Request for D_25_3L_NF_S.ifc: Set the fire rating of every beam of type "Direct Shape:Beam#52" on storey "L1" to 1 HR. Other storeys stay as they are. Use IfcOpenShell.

First a look at what the model holds.

```python
import ifcopenshell
import ifcopenshell.util.element

model = ifcopenshell.open("D_25_3L_NF_S.ifc")
print(model.schema)
storey = next(s for s in model.by_type("IfcBuildingStorey") if s.Name == "L1")
beams = [e for e in ifcopenshell.util.element.get_decomposition(storey) if e.is_a("IfcBeam")]
seen = {}
for e in beams:
    element_type = ifcopenshell.util.element.get_type(e)
    key = (element_type.Name if element_type != e and element_type else None, ifcopenshell.util.element.get_pset(e, "Pset_BeamCommon", "FireRating"))
    seen[key] = seen.get(key, 0) + 1
for (name, value), count in sorted(seen.items(), key=str):
    print(count, "x", name, "|", value)
```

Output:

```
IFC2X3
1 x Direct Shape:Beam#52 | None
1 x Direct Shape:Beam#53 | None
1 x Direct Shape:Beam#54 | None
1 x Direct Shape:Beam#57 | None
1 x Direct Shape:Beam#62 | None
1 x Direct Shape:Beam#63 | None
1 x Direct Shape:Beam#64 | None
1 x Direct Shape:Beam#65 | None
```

```python
import ifcopenshell
import ifcopenshell.api.pset
import ifcopenshell.util.element

model = ifcopenshell.open("D_25_3L_NF_S.ifc")

storey = next(s for s in model.by_type("IfcBuildingStorey") if s.Name == "L1")
beams = [e for e in ifcopenshell.util.element.get_decomposition(storey) if e.is_a("IfcBeam")]

count = 0
for e in beams:
    element_type = ifcopenshell.util.element.get_type(e)
    if element_type in (None, e) or element_type.Name != "Direct Shape:Beam#52":
        continue
    # add_pset returns the element's existing set when there is one.
    pset = ifcopenshell.api.pset.add_pset(model, product=e, name="Pset_BeamCommon")
    ifcopenshell.api.pset.edit_pset(model, pset=pset, properties={"FireRating": "1 HR"})
    count += 1

print(count, "beams updated")

model.write("D_25_3L_NF_S_rev.ifc")
```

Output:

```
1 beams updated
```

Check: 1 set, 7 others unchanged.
